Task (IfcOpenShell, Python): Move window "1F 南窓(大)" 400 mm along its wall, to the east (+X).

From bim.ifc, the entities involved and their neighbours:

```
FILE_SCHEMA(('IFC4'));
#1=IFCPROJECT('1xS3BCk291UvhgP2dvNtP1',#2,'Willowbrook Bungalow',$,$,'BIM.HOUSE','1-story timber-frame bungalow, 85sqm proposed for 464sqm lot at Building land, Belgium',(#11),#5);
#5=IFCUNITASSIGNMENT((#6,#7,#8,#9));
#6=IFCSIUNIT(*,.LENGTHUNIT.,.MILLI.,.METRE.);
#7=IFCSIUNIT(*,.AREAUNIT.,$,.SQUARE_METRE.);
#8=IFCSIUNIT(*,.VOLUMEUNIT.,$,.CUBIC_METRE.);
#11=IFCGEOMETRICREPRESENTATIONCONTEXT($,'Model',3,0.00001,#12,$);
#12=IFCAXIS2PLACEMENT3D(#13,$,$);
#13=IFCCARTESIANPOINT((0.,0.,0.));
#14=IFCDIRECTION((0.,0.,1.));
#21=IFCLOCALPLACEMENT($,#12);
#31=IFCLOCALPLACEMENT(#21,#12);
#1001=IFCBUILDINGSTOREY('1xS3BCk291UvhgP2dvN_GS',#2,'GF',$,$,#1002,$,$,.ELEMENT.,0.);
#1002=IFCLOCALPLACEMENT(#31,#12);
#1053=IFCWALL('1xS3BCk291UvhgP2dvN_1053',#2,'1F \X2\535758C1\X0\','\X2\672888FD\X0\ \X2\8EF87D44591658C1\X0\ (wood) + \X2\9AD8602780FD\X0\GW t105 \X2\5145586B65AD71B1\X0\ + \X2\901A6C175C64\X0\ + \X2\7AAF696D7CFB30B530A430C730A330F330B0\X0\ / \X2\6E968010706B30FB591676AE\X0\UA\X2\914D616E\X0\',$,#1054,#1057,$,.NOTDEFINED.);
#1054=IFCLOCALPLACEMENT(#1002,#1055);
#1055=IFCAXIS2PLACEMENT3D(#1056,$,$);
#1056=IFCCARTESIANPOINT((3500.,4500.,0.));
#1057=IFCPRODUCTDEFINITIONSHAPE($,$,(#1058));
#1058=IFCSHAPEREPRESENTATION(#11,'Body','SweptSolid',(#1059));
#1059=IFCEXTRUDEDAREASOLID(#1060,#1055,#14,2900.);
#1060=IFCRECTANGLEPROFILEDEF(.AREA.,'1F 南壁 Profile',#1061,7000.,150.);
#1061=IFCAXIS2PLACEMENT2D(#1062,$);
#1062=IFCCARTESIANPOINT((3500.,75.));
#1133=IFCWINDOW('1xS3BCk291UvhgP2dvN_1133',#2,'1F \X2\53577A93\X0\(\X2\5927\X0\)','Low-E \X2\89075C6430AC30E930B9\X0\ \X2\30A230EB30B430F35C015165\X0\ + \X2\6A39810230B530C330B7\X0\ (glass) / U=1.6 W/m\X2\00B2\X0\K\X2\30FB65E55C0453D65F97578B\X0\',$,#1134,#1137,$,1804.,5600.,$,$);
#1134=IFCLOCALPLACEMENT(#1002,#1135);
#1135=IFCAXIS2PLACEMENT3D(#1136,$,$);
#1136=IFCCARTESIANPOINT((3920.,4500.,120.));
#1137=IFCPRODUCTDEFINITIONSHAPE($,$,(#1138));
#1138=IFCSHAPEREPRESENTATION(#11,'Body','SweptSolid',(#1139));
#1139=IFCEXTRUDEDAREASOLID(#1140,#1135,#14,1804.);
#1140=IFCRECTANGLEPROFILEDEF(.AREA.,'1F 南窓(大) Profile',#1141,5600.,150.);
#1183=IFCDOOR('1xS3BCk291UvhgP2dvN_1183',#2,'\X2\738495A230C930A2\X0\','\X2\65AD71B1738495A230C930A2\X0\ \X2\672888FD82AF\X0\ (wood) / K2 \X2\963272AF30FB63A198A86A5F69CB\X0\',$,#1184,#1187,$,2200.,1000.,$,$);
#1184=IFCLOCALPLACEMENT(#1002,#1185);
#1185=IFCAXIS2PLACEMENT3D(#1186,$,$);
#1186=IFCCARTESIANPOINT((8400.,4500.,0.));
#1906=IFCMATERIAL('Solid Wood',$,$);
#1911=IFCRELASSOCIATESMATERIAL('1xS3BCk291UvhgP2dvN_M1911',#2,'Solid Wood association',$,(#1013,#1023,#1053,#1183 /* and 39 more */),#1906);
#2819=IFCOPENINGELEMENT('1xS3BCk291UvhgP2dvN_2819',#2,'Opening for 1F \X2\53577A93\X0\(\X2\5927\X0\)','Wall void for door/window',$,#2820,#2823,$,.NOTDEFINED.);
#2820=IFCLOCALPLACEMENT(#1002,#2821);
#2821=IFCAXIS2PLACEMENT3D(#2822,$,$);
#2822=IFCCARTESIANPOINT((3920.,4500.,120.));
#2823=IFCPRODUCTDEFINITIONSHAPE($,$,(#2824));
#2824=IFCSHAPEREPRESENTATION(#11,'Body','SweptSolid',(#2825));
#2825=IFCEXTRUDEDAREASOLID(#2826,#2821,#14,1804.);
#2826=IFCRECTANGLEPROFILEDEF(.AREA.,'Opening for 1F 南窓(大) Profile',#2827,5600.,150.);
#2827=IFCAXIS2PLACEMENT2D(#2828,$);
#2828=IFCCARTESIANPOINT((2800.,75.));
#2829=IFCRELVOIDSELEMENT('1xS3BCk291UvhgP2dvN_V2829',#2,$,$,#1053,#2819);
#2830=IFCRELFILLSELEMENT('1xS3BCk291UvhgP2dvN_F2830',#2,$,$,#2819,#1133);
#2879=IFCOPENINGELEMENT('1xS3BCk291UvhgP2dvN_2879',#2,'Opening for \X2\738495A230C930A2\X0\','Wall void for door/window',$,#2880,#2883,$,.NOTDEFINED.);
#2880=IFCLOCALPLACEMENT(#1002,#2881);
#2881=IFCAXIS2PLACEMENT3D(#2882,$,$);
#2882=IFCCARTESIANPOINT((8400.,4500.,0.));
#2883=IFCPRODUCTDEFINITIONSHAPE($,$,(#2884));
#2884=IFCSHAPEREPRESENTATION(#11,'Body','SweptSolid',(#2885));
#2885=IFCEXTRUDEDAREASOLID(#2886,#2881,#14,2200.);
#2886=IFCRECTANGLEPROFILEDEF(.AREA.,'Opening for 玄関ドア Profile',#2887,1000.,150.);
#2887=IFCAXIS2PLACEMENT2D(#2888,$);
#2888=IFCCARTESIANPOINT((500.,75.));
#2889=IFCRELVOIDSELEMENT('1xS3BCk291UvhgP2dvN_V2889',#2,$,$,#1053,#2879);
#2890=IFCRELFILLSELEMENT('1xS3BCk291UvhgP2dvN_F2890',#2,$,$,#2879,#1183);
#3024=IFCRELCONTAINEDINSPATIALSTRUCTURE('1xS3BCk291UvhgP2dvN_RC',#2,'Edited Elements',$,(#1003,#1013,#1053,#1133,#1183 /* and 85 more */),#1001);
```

```python
import ifcopenshell
import ifcopenshell.api.geometry
import ifcopenshell.util.placement

model = ifcopenshell.open("bim.ifc")

window = model.by_id(1133)
opening = window.FillsVoids[0].RelatingOpeningElement
wall = opening.VoidsElements[0].RelatingBuildingElement

wall_matrix = ifcopenshell.util.placement.get_local_placement(wall.ObjectPlacement)
shift = wall_matrix[:3, 0] * 400.0
before = ifcopenshell.util.placement.get_local_placement(window.ObjectPlacement)[:3, 3].copy()

# The window is not placed relative to its opening, so move both.
for product in (opening, window):
    matrix = ifcopenshell.util.placement.get_local_placement(product.ObjectPlacement)
    matrix[:3, 3] += shift
    ifcopenshell.api.geometry.edit_object_placement(model, product=product, matrix=matrix, is_si=False)

after = ifcopenshell.util.placement.get_local_placement(window.ObjectPlacement)[:3, 3]
print("window moved by", (after - before).round(3) + 0.0)

model.write("bim_updated.ifc")
```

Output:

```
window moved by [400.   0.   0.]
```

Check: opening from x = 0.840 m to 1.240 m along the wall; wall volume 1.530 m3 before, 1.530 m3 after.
